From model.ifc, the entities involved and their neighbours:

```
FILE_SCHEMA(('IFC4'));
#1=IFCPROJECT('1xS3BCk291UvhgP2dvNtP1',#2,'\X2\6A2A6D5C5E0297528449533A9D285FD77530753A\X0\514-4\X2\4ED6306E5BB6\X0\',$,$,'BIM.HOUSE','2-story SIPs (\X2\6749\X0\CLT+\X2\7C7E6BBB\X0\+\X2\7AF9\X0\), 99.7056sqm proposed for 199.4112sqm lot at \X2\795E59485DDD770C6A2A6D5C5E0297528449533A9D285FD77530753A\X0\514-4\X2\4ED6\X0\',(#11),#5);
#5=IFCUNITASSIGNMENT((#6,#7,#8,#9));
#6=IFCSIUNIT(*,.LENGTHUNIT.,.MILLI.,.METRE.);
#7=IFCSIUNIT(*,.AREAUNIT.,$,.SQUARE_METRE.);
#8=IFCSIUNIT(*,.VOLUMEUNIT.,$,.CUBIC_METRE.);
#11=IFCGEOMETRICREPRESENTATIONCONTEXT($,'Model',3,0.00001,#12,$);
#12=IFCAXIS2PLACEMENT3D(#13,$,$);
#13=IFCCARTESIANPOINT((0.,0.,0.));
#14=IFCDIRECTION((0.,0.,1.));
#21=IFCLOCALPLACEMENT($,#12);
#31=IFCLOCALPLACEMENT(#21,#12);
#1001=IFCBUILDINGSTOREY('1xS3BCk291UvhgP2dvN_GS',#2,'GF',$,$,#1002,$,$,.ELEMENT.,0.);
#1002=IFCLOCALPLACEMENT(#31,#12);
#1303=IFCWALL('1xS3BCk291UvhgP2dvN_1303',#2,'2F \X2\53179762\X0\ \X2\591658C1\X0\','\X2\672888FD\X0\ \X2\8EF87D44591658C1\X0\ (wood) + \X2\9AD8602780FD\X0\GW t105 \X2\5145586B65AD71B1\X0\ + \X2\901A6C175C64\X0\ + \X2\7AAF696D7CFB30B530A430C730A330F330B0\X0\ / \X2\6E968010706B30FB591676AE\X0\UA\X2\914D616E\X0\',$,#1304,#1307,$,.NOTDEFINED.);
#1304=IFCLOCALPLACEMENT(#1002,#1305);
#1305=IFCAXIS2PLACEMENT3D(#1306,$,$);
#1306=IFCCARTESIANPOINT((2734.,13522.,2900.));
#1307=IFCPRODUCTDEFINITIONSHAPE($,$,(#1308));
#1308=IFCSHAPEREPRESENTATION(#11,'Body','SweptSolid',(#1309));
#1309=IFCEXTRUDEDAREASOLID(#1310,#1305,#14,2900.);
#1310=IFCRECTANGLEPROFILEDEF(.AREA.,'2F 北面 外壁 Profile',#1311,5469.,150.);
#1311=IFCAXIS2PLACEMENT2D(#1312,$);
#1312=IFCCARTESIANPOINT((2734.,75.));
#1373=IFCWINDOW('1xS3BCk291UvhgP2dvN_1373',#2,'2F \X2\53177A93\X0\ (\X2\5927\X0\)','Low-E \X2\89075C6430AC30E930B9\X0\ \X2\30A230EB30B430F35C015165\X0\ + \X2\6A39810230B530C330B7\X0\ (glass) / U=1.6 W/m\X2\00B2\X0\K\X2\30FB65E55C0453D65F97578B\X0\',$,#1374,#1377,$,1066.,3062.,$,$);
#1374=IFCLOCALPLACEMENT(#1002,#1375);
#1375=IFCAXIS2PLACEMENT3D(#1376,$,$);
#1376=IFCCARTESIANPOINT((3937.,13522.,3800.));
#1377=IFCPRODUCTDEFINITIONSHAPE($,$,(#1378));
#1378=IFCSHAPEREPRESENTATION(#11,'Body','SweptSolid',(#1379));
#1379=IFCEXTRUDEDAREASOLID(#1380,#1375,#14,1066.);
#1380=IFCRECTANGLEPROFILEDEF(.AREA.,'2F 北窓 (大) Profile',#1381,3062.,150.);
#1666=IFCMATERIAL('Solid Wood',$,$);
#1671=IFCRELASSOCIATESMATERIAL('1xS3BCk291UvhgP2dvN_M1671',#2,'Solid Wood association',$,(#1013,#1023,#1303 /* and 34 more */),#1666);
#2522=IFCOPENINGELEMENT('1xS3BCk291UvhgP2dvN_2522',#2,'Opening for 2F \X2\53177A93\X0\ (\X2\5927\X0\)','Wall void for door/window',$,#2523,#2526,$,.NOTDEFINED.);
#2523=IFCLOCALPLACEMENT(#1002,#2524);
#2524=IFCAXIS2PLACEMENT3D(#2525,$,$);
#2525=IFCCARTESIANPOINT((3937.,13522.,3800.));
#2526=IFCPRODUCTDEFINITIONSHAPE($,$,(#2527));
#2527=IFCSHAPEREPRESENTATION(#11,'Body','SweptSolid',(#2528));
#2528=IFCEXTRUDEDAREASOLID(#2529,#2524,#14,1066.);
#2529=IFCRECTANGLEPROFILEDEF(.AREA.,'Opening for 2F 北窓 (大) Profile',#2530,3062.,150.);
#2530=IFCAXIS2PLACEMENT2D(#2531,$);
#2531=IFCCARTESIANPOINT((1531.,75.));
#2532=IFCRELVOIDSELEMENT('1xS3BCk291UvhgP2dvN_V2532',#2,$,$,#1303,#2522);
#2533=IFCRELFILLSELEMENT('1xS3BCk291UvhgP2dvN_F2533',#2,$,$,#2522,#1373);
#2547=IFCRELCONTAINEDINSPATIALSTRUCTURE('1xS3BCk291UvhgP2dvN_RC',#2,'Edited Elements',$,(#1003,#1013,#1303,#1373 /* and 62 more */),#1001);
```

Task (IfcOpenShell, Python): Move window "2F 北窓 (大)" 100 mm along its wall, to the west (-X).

```python
import ifcopenshell
import ifcopenshell.api.geometry
import ifcopenshell.util.placement
import ifcopenshell.util.unit

model = ifcopenshell.open("model.ifc")
unit_scale = ifcopenshell.util.unit.calculate_unit_scale(model)

window = model.by_id(1373)
opening = window.FillsVoids[0].RelatingOpeningElement
wall = opening.VoidsElements[0].RelatingBuildingElement

wall_matrix = ifcopenshell.util.placement.get_local_placement(wall.ObjectPlacement)
shift = wall_matrix[:3, 0] * -0.1 / unit_scale
before = ifcopenshell.util.placement.get_local_placement(window.ObjectPlacement)[:3, 3].copy()

# The window is not placed relative to its opening, so move both.
for product in (opening, window):
    matrix = ifcopenshell.util.placement.get_local_placement(product.ObjectPlacement)
    matrix[:3, 3] += shift
    ifcopenshell.api.geometry.edit_object_placement(model, product=product, matrix=matrix, is_si=False)

after = ifcopenshell.util.placement.get_local_placement(window.ObjectPlacement)[:3, 3]
print("window moved by", (after - before).round(3) + 0.0)

model.write("model_v2.ifc")
```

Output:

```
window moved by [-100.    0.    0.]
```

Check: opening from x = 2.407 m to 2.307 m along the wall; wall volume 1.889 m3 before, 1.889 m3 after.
